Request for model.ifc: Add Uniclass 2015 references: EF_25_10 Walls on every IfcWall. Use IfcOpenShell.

First a look at what the model holds.

```python
import ifcopenshell

model = ifcopenshell.open("model.ifc")
print(model.schema)
print("classifications:", [c.Name for c in model.by_type("IfcClassification")])
for ifc_class in ("IfcDoor", "IfcRoof", "IfcStair", "IfcWall", "IfcWindow"):
    print(ifc_class, len(model.by_type(ifc_class)))
```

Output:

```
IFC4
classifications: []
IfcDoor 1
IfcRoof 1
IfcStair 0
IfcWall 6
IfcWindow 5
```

```python
import ifcopenshell
import ifcopenshell.api.classification

model = ifcopenshell.open("model.ifc")

system = ifcopenshell.api.classification.add_classification(model, classification="Uniclass 2015")

codes = {
    "IfcWall": ("EF_25_10", "Walls"),
}
for ifc_class, (code, name) in codes.items():
    products = model.by_type(ifc_class)
    ifcopenshell.api.classification.add_reference(
        model, products=products, classification=system, identification=code, name=name
    )
    print(code, len(products))

model.write("model_rev.ifc")
```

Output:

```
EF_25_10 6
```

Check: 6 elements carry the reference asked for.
